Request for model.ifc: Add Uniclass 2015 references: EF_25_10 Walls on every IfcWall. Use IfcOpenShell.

First a look at what the model holds.

```python
import ifcopenshell

model = ifcopenshell.open("model.ifc")
print(model.schema)
print("classifications:", [c.Name for c in model.by_type("IfcClassification")])
for ifc_class in ("IfcDoor", "IfcRoof", "IfcStair", "IfcWall", "IfcWindow"):
    print(ifc_class, len(model.by_type(ifc_class)))
```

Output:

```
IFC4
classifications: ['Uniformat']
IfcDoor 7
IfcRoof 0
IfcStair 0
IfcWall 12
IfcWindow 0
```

```python
import ifcopenshell
import ifcopenshell.api.classification

model = ifcopenshell.open("model.ifc")

system = ifcopenshell.api.classification.add_classification(model, classification="Uniclass 2015")

codes = {
    "IfcWall": ("EF_25_10", "Walls"),
}
for ifc_class, (code, name) in codes.items():
    products = model.by_type(ifc_class)
    ifcopenshell.api.classification.add_reference(
        model, products=products, classification=system, identification=code, name=name
    )
    print(code, len(products))

model.write("model-out.ifc")
```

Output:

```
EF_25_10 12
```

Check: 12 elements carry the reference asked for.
